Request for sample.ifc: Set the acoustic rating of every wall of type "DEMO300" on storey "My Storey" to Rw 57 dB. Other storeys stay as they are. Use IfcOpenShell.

First a look at what the model holds.

```python
import ifcopenshell
import ifcopenshell.util.element

model = ifcopenshell.open("sample.ifc")
print(model.schema)
storey = next(s for s in model.by_type("IfcBuildingStorey") if s.Name == "My Storey")
walls = [e for e in ifcopenshell.util.element.get_decomposition(storey) if e.is_a("IfcWall")]
seen = {}
for e in walls:
    element_type = ifcopenshell.util.element.get_type(e)
    key = (element_type.Name if element_type != e and element_type else None, ifcopenshell.util.element.get_pset(e, "Pset_WallCommon", "AcousticRating"))
    seen[key] = seen.get(key, 0) + 1
for (name, value), count in sorted(seen.items(), key=str):
    print(count, "x", name, "|", value)
```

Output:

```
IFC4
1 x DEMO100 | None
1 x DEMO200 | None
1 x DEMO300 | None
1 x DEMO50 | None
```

```python
import ifcopenshell
import ifcopenshell.api.pset
import ifcopenshell.util.element

model = ifcopenshell.open("sample.ifc")

storey = next(s for s in model.by_type("IfcBuildingStorey") if s.Name == "My Storey")
walls = [e for e in ifcopenshell.util.element.get_decomposition(storey) if e.is_a("IfcWall")]

count = 0
for e in walls:
    element_type = ifcopenshell.util.element.get_type(e)
    if element_type in (None, e) or element_type.Name != "DEMO300":
        continue
    # add_pset returns the element's existing set when there is one.
    pset = ifcopenshell.api.pset.add_pset(model, product=e, name="Pset_WallCommon")
    ifcopenshell.api.pset.edit_pset(model, pset=pset, properties={"AcousticRating": "Rw 57 dB"})
    count += 1

print(count, "walls updated")

model.write("sample_rev.ifc")
```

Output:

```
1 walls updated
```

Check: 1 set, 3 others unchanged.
